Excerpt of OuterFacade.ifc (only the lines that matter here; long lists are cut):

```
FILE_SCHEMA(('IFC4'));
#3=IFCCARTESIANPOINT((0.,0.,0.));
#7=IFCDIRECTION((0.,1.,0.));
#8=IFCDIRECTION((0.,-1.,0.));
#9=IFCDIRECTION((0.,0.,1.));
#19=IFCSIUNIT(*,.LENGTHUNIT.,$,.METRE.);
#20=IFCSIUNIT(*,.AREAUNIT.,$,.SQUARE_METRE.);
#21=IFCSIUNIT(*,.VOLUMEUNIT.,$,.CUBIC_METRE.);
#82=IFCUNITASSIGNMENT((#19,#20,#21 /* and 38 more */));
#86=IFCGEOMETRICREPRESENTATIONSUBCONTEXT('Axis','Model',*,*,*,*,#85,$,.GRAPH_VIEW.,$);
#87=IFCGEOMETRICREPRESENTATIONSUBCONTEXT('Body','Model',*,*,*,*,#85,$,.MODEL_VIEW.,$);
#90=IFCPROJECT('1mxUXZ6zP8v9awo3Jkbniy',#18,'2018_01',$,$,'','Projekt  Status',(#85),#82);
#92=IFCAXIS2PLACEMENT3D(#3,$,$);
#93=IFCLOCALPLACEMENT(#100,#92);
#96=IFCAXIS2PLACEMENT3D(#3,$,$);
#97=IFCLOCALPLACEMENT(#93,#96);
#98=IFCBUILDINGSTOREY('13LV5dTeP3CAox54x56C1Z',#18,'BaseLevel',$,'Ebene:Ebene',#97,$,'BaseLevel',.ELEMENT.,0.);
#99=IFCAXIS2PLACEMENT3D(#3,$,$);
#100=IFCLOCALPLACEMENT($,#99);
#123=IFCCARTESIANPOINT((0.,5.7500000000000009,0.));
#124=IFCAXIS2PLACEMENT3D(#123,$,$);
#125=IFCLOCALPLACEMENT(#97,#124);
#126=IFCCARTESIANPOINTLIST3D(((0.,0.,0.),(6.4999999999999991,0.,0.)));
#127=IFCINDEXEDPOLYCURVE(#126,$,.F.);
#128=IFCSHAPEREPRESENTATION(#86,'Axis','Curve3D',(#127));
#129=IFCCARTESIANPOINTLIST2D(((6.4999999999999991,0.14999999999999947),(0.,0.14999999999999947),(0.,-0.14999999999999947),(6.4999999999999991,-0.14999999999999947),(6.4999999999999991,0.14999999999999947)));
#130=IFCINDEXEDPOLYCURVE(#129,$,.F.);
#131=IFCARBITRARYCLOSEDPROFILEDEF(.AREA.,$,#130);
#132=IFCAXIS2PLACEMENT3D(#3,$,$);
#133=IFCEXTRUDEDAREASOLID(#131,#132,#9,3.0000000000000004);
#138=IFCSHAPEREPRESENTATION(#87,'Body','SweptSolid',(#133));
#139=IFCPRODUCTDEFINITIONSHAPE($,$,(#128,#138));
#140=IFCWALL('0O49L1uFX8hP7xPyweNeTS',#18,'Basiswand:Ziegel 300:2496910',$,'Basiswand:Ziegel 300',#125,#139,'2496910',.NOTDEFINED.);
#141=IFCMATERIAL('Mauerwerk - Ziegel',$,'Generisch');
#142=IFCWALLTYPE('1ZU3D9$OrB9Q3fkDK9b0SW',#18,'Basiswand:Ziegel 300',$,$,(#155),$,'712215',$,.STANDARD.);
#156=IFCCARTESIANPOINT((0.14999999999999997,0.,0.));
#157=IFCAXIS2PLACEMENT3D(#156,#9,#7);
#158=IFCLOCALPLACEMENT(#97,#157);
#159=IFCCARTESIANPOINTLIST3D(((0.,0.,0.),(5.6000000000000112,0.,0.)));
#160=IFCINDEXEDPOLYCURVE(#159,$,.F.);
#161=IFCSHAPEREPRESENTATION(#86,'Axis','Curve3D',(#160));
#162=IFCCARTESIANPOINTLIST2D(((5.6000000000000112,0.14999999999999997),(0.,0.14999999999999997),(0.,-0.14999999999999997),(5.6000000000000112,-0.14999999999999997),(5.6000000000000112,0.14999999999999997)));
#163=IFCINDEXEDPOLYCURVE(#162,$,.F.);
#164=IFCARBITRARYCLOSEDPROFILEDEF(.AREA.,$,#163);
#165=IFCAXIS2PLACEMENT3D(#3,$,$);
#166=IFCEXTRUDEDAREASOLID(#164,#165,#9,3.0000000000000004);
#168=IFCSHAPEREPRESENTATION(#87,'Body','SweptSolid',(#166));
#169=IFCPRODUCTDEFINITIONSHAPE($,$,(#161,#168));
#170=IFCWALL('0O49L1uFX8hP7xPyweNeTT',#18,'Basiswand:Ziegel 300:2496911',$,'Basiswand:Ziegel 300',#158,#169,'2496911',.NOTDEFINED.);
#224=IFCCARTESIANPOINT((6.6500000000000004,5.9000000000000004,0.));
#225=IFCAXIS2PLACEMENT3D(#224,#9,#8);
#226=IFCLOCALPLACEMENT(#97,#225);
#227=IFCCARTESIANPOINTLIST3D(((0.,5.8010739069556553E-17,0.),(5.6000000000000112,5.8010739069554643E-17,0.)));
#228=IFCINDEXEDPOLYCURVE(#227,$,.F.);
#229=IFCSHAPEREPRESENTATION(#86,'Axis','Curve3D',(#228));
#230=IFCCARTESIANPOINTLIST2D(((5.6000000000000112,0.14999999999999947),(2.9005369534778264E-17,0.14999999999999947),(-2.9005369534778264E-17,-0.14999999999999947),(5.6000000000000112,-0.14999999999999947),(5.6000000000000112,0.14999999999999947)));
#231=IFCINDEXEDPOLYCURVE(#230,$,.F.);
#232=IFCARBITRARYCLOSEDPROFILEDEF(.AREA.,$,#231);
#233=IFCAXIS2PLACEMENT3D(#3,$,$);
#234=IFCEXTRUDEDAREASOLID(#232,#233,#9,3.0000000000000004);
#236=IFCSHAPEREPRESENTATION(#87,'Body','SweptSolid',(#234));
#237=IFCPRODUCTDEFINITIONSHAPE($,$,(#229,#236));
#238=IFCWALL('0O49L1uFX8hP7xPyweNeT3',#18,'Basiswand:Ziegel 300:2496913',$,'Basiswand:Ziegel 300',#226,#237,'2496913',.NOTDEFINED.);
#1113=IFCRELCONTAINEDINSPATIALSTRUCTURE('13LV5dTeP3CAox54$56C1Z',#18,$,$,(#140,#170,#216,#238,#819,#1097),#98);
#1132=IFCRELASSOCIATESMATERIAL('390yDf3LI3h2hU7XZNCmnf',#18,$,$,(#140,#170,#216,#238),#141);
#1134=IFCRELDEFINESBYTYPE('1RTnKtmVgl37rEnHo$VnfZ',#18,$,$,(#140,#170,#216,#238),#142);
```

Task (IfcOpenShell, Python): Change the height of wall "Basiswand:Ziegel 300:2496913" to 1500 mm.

```python
import ifcopenshell
import ifcopenshell.geom
import ifcopenshell.util.representation
import ifcopenshell.util.shape
import ifcopenshell.util.unit

model = ifcopenshell.open("OuterFacade.ifc")
unit_scale = ifcopenshell.util.unit.calculate_unit_scale(model)
settings = ifcopenshell.geom.settings()


def volume(element):
    """Net volume in cubic metres, openings subtracted."""
    shape = ifcopenshell.geom.create_shape(settings, element)
    return ifcopenshell.util.shape.get_volume(shape.geometry)


wall = model.by_guid("0O49L1uFX8hP7xPyweNeT3")
before = volume(wall)

body = ifcopenshell.util.representation.get_representation(wall, "Model", "Body")
solid = body.Items[0]
old_height = solid.Depth
solid.Depth = 1.5 / unit_scale
after = volume(wall)

print(f"height {old_height:g} -> {solid.Depth:g}, volume {before:.3f} -> {after:.3f} m3")

model.write("OuterFacade_rev.ifc")
```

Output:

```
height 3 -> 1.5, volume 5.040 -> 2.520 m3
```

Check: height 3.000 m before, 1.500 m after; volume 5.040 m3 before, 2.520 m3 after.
